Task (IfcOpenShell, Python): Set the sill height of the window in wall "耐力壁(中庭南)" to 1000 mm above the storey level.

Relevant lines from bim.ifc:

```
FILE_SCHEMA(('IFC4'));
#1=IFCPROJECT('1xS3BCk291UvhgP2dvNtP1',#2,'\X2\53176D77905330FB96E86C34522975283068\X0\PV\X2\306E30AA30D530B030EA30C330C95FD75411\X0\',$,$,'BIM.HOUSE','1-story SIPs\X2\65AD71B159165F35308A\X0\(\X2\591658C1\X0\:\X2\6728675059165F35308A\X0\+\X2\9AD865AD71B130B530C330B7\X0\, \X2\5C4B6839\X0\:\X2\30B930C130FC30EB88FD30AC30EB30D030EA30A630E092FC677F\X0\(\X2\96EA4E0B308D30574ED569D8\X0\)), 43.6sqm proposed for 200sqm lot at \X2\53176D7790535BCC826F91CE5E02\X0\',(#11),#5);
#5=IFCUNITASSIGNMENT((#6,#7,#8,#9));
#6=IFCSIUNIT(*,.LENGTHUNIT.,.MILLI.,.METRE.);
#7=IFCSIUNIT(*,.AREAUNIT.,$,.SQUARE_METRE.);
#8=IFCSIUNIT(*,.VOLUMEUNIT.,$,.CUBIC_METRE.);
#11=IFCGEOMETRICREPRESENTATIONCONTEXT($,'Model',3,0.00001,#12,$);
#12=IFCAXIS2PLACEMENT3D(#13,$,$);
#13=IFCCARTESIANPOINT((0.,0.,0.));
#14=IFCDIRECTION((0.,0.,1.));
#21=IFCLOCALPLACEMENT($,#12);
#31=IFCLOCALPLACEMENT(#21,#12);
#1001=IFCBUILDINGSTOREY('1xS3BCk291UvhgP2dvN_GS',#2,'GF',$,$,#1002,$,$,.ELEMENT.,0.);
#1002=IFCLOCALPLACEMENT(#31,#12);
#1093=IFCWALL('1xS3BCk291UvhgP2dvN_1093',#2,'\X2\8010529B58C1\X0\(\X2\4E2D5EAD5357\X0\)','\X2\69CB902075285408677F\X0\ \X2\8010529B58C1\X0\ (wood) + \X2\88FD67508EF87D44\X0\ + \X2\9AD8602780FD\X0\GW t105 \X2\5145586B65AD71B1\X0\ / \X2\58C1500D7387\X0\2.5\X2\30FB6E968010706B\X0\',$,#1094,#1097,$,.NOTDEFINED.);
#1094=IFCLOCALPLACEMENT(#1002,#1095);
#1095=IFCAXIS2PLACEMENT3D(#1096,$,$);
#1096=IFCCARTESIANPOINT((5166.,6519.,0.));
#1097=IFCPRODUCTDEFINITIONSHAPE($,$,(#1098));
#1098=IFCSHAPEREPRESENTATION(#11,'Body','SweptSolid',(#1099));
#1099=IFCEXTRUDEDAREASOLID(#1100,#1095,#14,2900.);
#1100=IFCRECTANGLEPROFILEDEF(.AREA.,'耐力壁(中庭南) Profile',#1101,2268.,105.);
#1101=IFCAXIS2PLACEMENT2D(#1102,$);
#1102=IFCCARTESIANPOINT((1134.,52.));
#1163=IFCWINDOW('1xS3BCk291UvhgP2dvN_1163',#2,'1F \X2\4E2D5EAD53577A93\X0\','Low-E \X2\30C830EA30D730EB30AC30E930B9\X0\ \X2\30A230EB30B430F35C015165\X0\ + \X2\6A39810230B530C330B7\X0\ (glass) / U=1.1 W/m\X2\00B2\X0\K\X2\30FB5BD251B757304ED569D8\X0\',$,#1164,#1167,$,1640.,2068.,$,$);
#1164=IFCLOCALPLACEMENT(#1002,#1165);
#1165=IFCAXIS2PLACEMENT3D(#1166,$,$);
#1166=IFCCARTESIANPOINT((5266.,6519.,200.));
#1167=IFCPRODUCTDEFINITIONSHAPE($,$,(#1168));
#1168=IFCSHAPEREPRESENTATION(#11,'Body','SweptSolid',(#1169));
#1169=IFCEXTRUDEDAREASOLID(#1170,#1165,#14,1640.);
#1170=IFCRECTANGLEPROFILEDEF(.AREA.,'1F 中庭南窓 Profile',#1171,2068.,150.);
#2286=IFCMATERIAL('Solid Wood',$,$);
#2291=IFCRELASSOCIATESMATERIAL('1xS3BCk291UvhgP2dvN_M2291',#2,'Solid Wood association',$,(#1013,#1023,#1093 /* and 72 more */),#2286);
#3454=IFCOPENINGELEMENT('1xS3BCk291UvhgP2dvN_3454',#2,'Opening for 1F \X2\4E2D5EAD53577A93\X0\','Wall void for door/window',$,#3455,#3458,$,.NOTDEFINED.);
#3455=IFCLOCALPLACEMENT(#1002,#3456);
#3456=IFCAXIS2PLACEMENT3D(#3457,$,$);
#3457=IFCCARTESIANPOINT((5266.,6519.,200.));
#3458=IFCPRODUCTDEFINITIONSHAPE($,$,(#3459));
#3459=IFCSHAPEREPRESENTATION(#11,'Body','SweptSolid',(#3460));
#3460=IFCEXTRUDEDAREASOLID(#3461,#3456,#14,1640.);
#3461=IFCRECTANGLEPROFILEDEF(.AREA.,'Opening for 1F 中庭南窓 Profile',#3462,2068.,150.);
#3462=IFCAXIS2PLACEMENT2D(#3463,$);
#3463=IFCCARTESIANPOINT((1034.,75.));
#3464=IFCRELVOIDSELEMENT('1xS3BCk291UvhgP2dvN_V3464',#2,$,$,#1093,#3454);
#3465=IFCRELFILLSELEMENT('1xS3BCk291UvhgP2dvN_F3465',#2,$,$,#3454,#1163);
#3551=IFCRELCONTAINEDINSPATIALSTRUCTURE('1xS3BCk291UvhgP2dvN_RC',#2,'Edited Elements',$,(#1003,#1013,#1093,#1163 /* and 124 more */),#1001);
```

```python
import numpy as np
import ifcopenshell
import ifcopenshell.api.geometry
import ifcopenshell.geom
import ifcopenshell.util.element
import ifcopenshell.util.placement
import ifcopenshell.util.shape
import ifcopenshell.util.unit

model = ifcopenshell.open("bim.ifc")
unit_scale = ifcopenshell.util.unit.calculate_unit_scale(model)

window = model.by_guid("1xS3BCk291UvhgP2dvN_1163")
opening = window.FillsVoids[0].RelatingOpeningElement
storey = ifcopenshell.util.element.get_container(window, ifc_class="IfcBuildingStorey")
level = ifcopenshell.util.placement.get_local_placement(storey.ObjectPlacement)[2, 3]

# The opening's origin need not be at the sill, so measure its lowest point.
shape = ifcopenshell.geom.create_shape(ifcopenshell.geom.settings(), opening)
bottom = ifcopenshell.util.shape.get_shape_bottom_elevation(shape, shape.geometry) / unit_scale
dz = level + 1 / unit_scale - bottom

shift = np.array([0.0, 0.0, dz])
# The window is not placed relative to its opening, so move both.
for product in (opening, window):
    matrix = ifcopenshell.util.placement.get_local_placement(product.ObjectPlacement)
    matrix[:3, 3] += shift
    ifcopenshell.api.geometry.edit_object_placement(model, product=product, matrix=matrix, is_si=False)

print(f"moved by {dz * unit_scale:+.3f} m")

model.write("bim_updated.ifc")
```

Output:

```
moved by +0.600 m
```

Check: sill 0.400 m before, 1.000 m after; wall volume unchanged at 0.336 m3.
